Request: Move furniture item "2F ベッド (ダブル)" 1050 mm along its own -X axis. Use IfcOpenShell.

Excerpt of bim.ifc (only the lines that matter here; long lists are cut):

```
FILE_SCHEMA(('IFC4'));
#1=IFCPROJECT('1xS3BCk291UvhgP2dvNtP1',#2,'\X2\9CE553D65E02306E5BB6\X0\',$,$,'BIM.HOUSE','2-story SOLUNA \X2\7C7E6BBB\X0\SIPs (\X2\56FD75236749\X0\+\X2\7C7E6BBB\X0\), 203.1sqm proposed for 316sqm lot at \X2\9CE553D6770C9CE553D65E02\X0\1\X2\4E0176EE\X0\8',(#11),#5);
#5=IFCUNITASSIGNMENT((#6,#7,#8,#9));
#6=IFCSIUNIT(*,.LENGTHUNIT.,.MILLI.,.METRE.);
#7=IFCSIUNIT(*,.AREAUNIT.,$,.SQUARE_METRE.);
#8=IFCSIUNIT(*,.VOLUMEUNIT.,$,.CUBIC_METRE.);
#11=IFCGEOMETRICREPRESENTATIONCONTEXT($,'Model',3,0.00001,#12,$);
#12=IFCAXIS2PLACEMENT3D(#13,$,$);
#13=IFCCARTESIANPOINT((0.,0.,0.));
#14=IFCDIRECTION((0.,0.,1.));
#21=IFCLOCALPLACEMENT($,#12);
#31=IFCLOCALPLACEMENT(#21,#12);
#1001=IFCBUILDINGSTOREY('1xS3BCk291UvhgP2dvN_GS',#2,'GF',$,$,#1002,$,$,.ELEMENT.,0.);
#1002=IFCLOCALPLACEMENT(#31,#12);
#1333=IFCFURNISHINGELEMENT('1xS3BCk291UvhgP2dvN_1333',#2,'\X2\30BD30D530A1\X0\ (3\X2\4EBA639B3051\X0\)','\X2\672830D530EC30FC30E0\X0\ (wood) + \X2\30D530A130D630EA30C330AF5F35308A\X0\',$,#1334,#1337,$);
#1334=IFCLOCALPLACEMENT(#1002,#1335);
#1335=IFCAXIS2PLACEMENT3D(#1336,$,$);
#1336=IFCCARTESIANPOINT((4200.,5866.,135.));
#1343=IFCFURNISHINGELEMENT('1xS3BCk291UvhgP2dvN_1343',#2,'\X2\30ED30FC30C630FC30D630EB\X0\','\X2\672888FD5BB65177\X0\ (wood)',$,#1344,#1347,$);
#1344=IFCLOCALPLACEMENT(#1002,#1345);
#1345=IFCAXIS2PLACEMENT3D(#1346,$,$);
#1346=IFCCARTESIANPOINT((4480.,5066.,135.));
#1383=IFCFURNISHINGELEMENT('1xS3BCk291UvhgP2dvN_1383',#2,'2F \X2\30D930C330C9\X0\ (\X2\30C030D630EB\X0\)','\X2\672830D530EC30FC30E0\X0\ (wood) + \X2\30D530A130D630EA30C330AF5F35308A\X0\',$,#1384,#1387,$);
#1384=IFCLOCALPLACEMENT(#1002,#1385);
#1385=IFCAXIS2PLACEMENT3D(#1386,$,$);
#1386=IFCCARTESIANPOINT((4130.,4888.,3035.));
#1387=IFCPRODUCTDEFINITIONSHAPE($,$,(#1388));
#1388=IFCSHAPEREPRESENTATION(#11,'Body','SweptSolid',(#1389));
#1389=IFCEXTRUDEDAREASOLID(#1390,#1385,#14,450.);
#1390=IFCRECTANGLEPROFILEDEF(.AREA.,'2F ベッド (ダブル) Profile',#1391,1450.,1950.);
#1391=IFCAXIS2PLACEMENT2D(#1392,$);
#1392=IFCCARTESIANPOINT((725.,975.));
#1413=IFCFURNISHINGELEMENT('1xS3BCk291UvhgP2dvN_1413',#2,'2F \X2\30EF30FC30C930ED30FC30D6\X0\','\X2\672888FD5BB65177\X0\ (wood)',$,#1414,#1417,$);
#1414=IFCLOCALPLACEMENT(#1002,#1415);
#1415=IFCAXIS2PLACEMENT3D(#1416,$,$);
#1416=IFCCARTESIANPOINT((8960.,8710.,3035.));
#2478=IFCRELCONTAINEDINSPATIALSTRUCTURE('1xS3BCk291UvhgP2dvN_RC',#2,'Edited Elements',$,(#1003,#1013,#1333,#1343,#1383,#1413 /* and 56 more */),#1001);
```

```python
import ifcopenshell
import ifcopenshell.api.geometry
import ifcopenshell.util.placement

model = ifcopenshell.open("bim.ifc")

item = model.by_guid("1xS3BCk291UvhgP2dvN_1383")
matrix = ifcopenshell.util.placement.get_local_placement(item.ObjectPlacement)
matrix[:3, 3] -= matrix[:3, 0] * 1050.0
ifcopenshell.api.geometry.edit_object_placement(model, product=item, matrix=matrix, is_si=False)

print(ifcopenshell.util.placement.get_local_placement(item.ObjectPlacement).round(3) + 0.0)

model.write("bim-out.ifc")
```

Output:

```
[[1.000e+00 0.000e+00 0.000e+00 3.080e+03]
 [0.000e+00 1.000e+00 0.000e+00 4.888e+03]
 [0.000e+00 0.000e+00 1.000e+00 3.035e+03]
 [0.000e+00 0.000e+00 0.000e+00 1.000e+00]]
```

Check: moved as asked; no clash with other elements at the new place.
